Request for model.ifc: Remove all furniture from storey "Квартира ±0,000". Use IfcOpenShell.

First a look at what the model holds.

```python
import ifcopenshell
import ifcopenshell.util.element

model = ifcopenshell.open("model.ifc")
print(model.schema)
storey = next(s for s in model.by_type("IfcBuildingStorey") if s.Name == "Квартира ±0,000")
furniture = [e for e in ifcopenshell.util.element.get_decomposition(storey) if e.is_a("IfcFurnishingElement")]
seen = {}
for e in furniture:
    element_type = ifcopenshell.util.element.get_type(e)
    name = element_type.Name if element_type not in (None, e) else None
    seen[name] = seen.get(name, 0) + 1
for name, count in sorted(seen.items(), key=str):
    print(count, "x", name)
```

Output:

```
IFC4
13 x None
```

```python
import ifcopenshell
import ifcopenshell.api.root
import ifcopenshell.util.element

model = ifcopenshell.open("model.ifc")

storey = next(s for s in model.by_type("IfcBuildingStorey") if s.Name == "Квартира ±0,000")
furniture = [e for e in ifcopenshell.util.element.get_decomposition(storey) if e.is_a("IfcFurnishingElement")]

for e in furniture:
    ifcopenshell.api.root.remove_product(model, product=e)
print(len(furniture), "removed")

model.write("model_updated.ifc")
```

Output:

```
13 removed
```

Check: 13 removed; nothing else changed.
